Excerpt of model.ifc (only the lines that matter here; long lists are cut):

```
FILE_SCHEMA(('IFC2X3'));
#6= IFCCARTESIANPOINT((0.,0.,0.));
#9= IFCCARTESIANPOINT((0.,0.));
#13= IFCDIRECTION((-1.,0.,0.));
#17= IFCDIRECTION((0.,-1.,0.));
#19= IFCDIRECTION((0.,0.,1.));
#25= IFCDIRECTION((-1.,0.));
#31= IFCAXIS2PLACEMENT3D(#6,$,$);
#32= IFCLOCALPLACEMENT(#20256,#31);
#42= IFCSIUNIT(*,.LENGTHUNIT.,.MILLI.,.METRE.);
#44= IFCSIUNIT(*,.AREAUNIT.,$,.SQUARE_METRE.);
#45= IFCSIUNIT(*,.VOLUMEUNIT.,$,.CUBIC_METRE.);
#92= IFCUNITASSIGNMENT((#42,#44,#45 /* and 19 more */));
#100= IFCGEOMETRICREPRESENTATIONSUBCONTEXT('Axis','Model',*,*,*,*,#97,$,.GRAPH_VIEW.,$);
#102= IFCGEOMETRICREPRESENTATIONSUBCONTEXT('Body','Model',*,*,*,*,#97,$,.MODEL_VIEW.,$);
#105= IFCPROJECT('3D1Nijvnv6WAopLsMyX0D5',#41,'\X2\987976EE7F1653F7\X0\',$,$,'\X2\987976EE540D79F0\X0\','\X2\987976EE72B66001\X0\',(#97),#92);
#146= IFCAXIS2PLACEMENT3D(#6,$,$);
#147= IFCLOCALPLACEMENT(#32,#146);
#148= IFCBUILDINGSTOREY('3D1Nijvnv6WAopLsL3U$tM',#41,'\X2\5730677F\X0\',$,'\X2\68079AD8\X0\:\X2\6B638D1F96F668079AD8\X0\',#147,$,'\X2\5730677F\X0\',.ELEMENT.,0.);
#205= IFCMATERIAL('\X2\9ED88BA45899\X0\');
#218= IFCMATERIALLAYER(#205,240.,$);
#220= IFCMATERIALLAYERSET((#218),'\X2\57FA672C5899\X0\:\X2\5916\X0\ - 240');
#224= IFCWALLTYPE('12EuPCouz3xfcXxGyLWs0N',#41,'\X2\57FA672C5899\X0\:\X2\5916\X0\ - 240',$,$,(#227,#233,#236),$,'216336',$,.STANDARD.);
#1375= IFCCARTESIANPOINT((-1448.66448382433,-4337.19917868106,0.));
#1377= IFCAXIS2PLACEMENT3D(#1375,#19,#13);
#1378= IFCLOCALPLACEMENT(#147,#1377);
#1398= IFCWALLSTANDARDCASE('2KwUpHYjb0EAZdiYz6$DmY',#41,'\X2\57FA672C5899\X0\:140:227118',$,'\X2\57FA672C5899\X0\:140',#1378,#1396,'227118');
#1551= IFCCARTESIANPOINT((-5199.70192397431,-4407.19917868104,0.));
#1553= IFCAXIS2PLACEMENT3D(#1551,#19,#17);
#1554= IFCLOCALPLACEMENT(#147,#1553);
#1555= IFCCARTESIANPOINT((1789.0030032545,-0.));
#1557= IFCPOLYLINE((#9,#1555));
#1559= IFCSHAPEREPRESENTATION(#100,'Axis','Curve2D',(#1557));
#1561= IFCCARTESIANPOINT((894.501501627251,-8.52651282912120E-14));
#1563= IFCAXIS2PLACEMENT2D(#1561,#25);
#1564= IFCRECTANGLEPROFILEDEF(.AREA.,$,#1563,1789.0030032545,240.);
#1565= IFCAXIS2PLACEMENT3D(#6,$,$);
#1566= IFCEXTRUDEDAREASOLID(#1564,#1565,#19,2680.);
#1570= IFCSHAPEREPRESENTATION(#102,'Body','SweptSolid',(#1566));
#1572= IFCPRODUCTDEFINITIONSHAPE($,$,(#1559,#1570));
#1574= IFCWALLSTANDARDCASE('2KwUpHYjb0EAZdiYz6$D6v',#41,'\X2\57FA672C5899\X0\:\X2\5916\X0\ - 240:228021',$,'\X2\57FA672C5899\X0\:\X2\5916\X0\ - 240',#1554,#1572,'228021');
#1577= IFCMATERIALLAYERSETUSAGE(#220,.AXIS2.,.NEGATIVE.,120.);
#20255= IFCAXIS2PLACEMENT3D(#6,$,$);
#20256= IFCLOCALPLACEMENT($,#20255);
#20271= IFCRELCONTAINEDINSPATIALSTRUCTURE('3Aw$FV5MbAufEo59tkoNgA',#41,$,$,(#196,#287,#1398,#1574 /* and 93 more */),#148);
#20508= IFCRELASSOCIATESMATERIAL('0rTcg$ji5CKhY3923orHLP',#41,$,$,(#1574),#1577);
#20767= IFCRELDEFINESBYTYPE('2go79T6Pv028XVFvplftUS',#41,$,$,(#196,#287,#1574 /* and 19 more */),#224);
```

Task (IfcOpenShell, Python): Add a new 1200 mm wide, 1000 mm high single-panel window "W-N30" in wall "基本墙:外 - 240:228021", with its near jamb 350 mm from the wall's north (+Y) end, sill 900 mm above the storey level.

```python
import numpy as np
import ifcopenshell
import ifcopenshell.api.feature
import ifcopenshell.api.geometry
import ifcopenshell.api.root
import ifcopenshell.api.spatial
import ifcopenshell.api.type
import ifcopenshell.geom
import ifcopenshell.util.element
import ifcopenshell.util.placement
import ifcopenshell.util.representation
import ifcopenshell.util.shape
import ifcopenshell.util.unit

model = ifcopenshell.open("model.ifc")
unit_scale = ifcopenshell.util.unit.calculate_unit_scale(model)
settings = ifcopenshell.geom.settings()


def volume(element):
    """Net volume in cubic metres, openings subtracted."""
    shape = ifcopenshell.geom.create_shape(settings, element)
    return ifcopenshell.util.shape.get_volume(shape.geometry)


wall = model.by_guid("2KwUpHYjb0EAZdiYz6$D6v")
storey = ifcopenshell.util.element.get_container(wall, ifc_class="IfcBuildingStorey")
context = ifcopenshell.util.representation.get_context(model, "Model", "Body", "MODEL_VIEW")
before = volume(wall)

width, height, from_end, sill = 1.2, 1, 0.35, 0.9  # metres

# The wall runs along its own X axis, and the end named is its -X end.
wall_shape = ifcopenshell.geom.create_shape(settings, wall)
x, y, z = ifcopenshell.util.shape.get_vertices(wall_shape.geometry).T
start = x.min() + from_end
face, thickness = float(y.min()), float(y.max() - y.min())
wall_matrix = ifcopenshell.util.placement.get_local_placement(wall.ObjectPlacement)
level = ifcopenshell.util.placement.get_local_placement(storey.ObjectPlacement)[2, 3]


def in_wall(x, y):
    """Placement at x, y metres in the wall's axes, at sill height."""
    matrix = wall_matrix.copy()
    matrix[:, 3] = wall_matrix @ np.array([x / unit_scale, y / unit_scale, 0.0, 1.0])
    matrix[2, 3] = level + sill / unit_scale
    return matrix


# Opening: a box that overshoots both wall faces by 50 mm.
opening = ifcopenshell.api.root.create_entity(model, ifc_class="IfcOpeningElement")
box = ifcopenshell.api.geometry.add_wall_representation(
    model, context=context, length=width, height=height, thickness=thickness + 0.1
)
ifcopenshell.api.geometry.assign_representation(model, product=opening, representation=box)
ifcopenshell.api.geometry.edit_object_placement(model, product=opening, matrix=in_wall(start, face - 0.05), is_si=False)
ifcopenshell.api.feature.add_feature(model, feature=opening, element=wall)

window = ifcopenshell.api.root.create_entity(model, ifc_class="IfcWindow", name="W-N30")
window.OverallWidth, window.OverallHeight = width / unit_scale, height / unit_scale
body = ifcopenshell.api.geometry.add_window_representation(
    model,
    context=context,
    overall_width=window.OverallWidth,
    overall_height=window.OverallHeight,
    partition_type="SINGLE_PANEL",
)
ifcopenshell.api.geometry.assign_representation(model, product=window, representation=body)
ifcopenshell.api.spatial.assign_container(model, products=[window], relating_structure=storey)
fills = ifcopenshell.api.feature.add_filling(model, opening=opening, element=window)
fills.OwnerHistory = window.OwnerHistory  # required in IFC2X3

# IFC2X3 keeps the operation on the window style.
style = ifcopenshell.api.root.create_entity(model, ifc_class="IfcWindowStyle", name="W-N30")
style.OperationType, style.ConstructionType = "SINGLE_PANEL", "NOTDEFINED"
style.ParameterTakesPrecedence = style.Sizeable = False
ifcopenshell.api.type.assign_type(model, related_objects=[window], relating_type=style)

# Centre the window in the wall's thickness.
ifcopenshell.api.geometry.edit_object_placement(model, product=window, matrix=in_wall(start, face), is_si=False)
window_shape = ifcopenshell.geom.create_shape(settings, window)
depth = ifcopenshell.util.shape.get_vertices(window_shape.geometry)[:, 1]
offset = face + thickness / 2 - (depth.min() + depth.max()) / 2
ifcopenshell.api.geometry.edit_object_placement(model, product=window, matrix=in_wall(start, offset), is_si=False)

after = volume(wall)

print(f"wall volume {before:.3f} -> {after:.3f} m3")

model.write("model_edited.ifc")
```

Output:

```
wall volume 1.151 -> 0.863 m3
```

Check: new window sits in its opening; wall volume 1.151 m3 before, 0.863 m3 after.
